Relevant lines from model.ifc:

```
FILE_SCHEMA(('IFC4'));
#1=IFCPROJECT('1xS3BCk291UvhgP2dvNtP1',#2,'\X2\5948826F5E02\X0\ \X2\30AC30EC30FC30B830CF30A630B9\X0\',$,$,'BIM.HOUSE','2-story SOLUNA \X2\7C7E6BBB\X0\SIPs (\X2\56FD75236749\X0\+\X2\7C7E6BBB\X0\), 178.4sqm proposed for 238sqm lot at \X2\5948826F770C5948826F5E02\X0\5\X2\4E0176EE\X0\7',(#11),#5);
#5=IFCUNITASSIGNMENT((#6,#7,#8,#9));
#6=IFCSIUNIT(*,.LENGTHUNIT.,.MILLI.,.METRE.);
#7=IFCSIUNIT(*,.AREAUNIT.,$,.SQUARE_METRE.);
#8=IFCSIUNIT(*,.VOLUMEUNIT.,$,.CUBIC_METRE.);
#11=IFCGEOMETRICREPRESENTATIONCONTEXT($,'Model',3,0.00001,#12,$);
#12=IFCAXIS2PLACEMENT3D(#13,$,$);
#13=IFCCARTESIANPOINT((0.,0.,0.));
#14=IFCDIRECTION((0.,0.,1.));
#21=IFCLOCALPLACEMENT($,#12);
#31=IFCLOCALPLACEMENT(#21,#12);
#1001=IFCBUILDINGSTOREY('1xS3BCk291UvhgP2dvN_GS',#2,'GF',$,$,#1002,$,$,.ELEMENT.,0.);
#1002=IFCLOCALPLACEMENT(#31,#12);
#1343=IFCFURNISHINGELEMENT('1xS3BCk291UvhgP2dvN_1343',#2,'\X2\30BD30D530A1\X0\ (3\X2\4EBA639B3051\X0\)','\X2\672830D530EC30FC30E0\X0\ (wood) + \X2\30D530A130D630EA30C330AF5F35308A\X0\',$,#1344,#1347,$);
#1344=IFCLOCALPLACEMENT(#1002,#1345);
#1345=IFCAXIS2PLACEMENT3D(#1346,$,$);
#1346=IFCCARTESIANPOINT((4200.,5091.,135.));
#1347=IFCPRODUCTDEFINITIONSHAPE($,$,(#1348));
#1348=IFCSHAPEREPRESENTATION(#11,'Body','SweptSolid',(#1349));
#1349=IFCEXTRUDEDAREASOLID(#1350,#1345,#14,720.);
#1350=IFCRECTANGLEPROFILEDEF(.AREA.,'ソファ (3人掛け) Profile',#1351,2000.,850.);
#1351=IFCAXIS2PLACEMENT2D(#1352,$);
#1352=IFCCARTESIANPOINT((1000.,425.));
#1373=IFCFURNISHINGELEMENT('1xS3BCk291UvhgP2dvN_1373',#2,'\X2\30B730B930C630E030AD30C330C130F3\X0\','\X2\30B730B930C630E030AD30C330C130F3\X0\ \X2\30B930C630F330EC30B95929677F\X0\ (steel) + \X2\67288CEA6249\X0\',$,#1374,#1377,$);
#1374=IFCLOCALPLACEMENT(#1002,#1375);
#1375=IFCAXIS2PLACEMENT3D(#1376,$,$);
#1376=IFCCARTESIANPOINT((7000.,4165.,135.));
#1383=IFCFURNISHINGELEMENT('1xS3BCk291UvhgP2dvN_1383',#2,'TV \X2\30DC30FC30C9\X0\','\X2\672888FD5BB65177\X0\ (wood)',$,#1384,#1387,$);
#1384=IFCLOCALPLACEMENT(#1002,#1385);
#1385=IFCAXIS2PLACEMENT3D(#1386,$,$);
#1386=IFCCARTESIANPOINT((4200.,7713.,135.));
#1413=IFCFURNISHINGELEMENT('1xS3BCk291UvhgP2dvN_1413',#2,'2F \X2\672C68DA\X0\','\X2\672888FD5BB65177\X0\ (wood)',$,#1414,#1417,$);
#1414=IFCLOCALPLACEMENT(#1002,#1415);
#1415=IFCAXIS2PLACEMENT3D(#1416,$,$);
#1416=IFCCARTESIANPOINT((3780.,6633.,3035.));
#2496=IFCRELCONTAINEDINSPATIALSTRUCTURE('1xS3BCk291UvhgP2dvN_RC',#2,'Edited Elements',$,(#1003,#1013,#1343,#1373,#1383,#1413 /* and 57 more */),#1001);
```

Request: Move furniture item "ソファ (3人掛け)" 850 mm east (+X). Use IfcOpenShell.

```python
import ifcopenshell
import ifcopenshell.api.geometry
import ifcopenshell.util.placement

model = ifcopenshell.open("model.ifc")

item = model.by_id(1343)
matrix = ifcopenshell.util.placement.get_local_placement(item.ObjectPlacement)
matrix[0, 3] += 850.0
ifcopenshell.api.geometry.edit_object_placement(model, product=item, matrix=matrix, is_si=False)

print(ifcopenshell.util.placement.get_local_placement(item.ObjectPlacement).round(3) + 0.0)

model.write("model_edited.ifc")
```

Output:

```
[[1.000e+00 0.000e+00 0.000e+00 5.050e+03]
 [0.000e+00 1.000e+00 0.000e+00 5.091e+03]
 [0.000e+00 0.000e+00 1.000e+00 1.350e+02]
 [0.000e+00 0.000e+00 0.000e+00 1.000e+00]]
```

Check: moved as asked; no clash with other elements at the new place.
